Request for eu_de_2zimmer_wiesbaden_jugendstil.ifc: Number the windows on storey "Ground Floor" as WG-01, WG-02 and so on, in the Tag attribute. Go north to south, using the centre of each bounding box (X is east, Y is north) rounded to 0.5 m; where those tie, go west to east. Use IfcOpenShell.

First a look at what the model holds.

```python
import ifcopenshell
import ifcopenshell.util.element
import ifcopenshell.util.placement

model = ifcopenshell.open("eu_de_2zimmer_wiesbaden_jugendstil.ifc")
print(model.schema)
storey = next(s for s in model.by_type("IfcBuildingStorey") if s.Name == "Ground Floor")
windows = [e for e in ifcopenshell.util.element.get_decomposition(storey) if e.is_a("IfcWindow")]
for e in sorted(windows, key=lambda e: e.id()):
    origin = ifcopenshell.util.placement.get_local_placement(e.ObjectPlacement)[:3, 3]
    print(e.id(), e.Tag, e.Name, origin.round(2) + 0.0, sep=" | ")
```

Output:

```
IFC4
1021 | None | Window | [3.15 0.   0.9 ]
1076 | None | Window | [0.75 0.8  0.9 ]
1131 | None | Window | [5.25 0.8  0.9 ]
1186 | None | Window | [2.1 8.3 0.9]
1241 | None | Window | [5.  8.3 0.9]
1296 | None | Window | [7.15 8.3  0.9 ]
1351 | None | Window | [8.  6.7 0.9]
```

```python
import ifcopenshell
import ifcopenshell.geom
import ifcopenshell.util.element
import ifcopenshell.util.shape

model = ifcopenshell.open("eu_de_2zimmer_wiesbaden_jugendstil.ifc")
settings = ifcopenshell.geom.settings()
settings.set("use-world-coords", True)


def centre(element):
    shape = ifcopenshell.geom.create_shape(settings, element)
    return ifcopenshell.util.shape.get_bbox_centroid(shape.geometry)


storey = next(s for s in model.by_type("IfcBuildingStorey") if s.Name == "Ground Floor")
windows = [e for e in ifcopenshell.util.element.get_decomposition(storey) if e.is_a("IfcWindow")]

# Insertion points can sit at a corner or the storey origin, so sort by the geometry (in metres).
centres = {e: centre(e) for e in windows}
windows.sort(key=lambda e: (-round(centres[e][1] / 0.5), centres[e][0]))

for i, e in enumerate(windows, start=1):
    number = f"WG-{i:02d}"
    e.Tag = number
    print(e.id(), number)

model.write("eu_de_2zimmer_wiesbaden_jugendstil_rev.ifc")
```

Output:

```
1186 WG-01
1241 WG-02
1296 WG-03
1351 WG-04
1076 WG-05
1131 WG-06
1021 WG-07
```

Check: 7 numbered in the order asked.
